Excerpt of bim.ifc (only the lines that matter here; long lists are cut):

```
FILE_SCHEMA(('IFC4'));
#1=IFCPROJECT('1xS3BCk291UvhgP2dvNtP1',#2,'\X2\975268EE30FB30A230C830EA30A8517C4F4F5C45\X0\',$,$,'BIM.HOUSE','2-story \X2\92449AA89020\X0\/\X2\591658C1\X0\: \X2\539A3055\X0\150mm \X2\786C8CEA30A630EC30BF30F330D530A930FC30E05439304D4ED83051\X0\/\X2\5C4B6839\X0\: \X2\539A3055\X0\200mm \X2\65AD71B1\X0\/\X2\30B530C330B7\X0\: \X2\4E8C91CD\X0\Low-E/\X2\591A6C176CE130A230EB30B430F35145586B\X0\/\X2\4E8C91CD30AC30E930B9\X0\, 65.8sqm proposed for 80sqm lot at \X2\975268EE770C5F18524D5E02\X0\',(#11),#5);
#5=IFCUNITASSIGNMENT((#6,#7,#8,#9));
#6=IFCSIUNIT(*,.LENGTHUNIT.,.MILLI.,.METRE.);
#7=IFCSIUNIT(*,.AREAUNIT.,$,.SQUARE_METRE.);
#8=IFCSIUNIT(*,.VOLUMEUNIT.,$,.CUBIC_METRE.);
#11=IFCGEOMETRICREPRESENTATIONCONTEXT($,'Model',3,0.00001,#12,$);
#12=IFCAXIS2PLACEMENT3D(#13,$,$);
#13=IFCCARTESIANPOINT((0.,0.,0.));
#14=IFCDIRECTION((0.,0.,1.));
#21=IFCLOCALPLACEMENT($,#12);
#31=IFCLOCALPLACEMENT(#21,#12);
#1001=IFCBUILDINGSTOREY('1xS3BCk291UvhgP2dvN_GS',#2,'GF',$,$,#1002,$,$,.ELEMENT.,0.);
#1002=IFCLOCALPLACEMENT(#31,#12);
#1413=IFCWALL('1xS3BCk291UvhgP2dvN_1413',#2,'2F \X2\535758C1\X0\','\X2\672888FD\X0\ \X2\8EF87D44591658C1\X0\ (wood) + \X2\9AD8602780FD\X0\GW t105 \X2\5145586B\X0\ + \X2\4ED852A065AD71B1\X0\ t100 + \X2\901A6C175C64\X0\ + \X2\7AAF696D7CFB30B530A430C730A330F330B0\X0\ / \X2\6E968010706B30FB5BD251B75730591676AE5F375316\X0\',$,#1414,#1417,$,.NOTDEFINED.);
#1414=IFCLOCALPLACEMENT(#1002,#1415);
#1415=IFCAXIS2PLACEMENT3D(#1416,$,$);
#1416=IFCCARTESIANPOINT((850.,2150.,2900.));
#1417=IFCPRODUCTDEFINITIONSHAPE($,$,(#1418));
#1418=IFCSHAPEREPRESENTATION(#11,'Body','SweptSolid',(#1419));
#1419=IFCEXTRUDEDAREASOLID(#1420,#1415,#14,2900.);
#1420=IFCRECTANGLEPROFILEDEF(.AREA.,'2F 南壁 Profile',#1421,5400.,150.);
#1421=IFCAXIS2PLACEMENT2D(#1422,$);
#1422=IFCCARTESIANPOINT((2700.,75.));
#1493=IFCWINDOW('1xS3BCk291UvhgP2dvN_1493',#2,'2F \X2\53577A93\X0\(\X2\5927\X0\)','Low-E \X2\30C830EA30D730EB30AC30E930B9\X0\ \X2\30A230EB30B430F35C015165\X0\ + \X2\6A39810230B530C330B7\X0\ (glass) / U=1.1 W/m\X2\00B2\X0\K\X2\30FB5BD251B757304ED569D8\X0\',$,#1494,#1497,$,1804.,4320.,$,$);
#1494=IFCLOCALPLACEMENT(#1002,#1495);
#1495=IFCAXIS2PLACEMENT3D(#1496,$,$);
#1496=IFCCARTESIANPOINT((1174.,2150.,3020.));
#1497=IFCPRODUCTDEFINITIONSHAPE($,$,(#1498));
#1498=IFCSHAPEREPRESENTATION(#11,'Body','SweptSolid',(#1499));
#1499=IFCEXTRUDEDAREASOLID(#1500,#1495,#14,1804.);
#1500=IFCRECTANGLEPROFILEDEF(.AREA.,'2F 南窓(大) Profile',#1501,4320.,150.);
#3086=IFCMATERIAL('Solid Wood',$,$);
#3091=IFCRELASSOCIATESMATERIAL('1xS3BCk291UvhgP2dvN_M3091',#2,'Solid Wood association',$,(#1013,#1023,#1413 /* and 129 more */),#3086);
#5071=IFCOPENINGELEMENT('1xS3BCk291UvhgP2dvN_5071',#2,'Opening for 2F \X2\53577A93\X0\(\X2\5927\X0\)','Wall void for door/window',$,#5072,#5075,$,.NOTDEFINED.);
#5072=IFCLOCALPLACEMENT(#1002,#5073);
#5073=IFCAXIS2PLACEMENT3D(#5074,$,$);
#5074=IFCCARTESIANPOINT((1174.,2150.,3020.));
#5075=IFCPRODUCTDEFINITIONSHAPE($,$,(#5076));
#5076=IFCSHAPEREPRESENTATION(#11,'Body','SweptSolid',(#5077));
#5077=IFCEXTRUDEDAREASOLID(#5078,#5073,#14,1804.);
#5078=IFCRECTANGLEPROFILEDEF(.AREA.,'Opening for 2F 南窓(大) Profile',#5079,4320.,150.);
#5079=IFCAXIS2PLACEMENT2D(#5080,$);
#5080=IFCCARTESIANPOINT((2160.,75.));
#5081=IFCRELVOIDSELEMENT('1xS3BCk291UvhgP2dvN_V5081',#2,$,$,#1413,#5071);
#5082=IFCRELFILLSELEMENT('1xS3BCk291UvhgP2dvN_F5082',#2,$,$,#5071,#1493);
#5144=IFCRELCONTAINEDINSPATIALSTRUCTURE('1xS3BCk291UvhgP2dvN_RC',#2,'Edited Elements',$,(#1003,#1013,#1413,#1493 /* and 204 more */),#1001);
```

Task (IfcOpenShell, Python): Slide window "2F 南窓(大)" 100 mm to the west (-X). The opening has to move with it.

```python
import ifcopenshell
import ifcopenshell.api.geometry
import ifcopenshell.util.placement
import ifcopenshell.util.unit

model = ifcopenshell.open("bim.ifc")
unit_scale = ifcopenshell.util.unit.calculate_unit_scale(model)

window = model.by_guid("1xS3BCk291UvhgP2dvN_1493")
opening = window.FillsVoids[0].RelatingOpeningElement
wall = opening.VoidsElements[0].RelatingBuildingElement

wall_matrix = ifcopenshell.util.placement.get_local_placement(wall.ObjectPlacement)
shift = wall_matrix[:3, 0] * -0.1 / unit_scale
before = ifcopenshell.util.placement.get_local_placement(window.ObjectPlacement)[:3, 3].copy()

# The window is not placed relative to its opening, so move both.
for product in (opening, window):
    matrix = ifcopenshell.util.placement.get_local_placement(product.ObjectPlacement)
    matrix[:3, 3] += shift
    ifcopenshell.api.geometry.edit_object_placement(model, product=product, matrix=matrix, is_si=False)

after = ifcopenshell.util.placement.get_local_placement(window.ObjectPlacement)[:3, 3]
print("window moved by", (after - before).round(3) + 0.0)

model.write("bim_v2.ifc")
```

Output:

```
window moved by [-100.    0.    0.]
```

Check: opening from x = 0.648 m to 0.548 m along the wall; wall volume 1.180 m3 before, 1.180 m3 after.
